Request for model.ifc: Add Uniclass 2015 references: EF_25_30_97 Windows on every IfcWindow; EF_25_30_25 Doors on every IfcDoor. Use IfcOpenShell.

First a look at what the model holds.

```python
import ifcopenshell

model = ifcopenshell.open("model.ifc")
print(model.schema)
print("classifications:", [c.Name for c in model.by_type("IfcClassification")])
for ifc_class in ("IfcDoor", "IfcRoof", "IfcStair", "IfcWall", "IfcWindow"):
    print(ifc_class, len(model.by_type(ifc_class)))
```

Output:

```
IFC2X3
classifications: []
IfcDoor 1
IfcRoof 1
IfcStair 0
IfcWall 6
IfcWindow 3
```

```python
import ifcopenshell
import ifcopenshell.api.classification

model = ifcopenshell.open("model.ifc")

# IFC2X3 requires Source and Edition and has no link from the project to the system.
system = model.create_entity("IfcClassification", Source="NBS", Edition="2015", Name="Uniclass 2015")

codes = {
    "IfcWindow": ("EF_25_30_97", "Windows"),
    "IfcDoor": ("EF_25_30_25", "Doors"),
}
for ifc_class, (code, name) in codes.items():
    products = model.by_type(ifc_class)
    ifcopenshell.api.classification.add_reference(
        model, products=products, classification=system, identification=code, name=name
    )
    print(code, len(products))

model.write("model_edited.ifc")
```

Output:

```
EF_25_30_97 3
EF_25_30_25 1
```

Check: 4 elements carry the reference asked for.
